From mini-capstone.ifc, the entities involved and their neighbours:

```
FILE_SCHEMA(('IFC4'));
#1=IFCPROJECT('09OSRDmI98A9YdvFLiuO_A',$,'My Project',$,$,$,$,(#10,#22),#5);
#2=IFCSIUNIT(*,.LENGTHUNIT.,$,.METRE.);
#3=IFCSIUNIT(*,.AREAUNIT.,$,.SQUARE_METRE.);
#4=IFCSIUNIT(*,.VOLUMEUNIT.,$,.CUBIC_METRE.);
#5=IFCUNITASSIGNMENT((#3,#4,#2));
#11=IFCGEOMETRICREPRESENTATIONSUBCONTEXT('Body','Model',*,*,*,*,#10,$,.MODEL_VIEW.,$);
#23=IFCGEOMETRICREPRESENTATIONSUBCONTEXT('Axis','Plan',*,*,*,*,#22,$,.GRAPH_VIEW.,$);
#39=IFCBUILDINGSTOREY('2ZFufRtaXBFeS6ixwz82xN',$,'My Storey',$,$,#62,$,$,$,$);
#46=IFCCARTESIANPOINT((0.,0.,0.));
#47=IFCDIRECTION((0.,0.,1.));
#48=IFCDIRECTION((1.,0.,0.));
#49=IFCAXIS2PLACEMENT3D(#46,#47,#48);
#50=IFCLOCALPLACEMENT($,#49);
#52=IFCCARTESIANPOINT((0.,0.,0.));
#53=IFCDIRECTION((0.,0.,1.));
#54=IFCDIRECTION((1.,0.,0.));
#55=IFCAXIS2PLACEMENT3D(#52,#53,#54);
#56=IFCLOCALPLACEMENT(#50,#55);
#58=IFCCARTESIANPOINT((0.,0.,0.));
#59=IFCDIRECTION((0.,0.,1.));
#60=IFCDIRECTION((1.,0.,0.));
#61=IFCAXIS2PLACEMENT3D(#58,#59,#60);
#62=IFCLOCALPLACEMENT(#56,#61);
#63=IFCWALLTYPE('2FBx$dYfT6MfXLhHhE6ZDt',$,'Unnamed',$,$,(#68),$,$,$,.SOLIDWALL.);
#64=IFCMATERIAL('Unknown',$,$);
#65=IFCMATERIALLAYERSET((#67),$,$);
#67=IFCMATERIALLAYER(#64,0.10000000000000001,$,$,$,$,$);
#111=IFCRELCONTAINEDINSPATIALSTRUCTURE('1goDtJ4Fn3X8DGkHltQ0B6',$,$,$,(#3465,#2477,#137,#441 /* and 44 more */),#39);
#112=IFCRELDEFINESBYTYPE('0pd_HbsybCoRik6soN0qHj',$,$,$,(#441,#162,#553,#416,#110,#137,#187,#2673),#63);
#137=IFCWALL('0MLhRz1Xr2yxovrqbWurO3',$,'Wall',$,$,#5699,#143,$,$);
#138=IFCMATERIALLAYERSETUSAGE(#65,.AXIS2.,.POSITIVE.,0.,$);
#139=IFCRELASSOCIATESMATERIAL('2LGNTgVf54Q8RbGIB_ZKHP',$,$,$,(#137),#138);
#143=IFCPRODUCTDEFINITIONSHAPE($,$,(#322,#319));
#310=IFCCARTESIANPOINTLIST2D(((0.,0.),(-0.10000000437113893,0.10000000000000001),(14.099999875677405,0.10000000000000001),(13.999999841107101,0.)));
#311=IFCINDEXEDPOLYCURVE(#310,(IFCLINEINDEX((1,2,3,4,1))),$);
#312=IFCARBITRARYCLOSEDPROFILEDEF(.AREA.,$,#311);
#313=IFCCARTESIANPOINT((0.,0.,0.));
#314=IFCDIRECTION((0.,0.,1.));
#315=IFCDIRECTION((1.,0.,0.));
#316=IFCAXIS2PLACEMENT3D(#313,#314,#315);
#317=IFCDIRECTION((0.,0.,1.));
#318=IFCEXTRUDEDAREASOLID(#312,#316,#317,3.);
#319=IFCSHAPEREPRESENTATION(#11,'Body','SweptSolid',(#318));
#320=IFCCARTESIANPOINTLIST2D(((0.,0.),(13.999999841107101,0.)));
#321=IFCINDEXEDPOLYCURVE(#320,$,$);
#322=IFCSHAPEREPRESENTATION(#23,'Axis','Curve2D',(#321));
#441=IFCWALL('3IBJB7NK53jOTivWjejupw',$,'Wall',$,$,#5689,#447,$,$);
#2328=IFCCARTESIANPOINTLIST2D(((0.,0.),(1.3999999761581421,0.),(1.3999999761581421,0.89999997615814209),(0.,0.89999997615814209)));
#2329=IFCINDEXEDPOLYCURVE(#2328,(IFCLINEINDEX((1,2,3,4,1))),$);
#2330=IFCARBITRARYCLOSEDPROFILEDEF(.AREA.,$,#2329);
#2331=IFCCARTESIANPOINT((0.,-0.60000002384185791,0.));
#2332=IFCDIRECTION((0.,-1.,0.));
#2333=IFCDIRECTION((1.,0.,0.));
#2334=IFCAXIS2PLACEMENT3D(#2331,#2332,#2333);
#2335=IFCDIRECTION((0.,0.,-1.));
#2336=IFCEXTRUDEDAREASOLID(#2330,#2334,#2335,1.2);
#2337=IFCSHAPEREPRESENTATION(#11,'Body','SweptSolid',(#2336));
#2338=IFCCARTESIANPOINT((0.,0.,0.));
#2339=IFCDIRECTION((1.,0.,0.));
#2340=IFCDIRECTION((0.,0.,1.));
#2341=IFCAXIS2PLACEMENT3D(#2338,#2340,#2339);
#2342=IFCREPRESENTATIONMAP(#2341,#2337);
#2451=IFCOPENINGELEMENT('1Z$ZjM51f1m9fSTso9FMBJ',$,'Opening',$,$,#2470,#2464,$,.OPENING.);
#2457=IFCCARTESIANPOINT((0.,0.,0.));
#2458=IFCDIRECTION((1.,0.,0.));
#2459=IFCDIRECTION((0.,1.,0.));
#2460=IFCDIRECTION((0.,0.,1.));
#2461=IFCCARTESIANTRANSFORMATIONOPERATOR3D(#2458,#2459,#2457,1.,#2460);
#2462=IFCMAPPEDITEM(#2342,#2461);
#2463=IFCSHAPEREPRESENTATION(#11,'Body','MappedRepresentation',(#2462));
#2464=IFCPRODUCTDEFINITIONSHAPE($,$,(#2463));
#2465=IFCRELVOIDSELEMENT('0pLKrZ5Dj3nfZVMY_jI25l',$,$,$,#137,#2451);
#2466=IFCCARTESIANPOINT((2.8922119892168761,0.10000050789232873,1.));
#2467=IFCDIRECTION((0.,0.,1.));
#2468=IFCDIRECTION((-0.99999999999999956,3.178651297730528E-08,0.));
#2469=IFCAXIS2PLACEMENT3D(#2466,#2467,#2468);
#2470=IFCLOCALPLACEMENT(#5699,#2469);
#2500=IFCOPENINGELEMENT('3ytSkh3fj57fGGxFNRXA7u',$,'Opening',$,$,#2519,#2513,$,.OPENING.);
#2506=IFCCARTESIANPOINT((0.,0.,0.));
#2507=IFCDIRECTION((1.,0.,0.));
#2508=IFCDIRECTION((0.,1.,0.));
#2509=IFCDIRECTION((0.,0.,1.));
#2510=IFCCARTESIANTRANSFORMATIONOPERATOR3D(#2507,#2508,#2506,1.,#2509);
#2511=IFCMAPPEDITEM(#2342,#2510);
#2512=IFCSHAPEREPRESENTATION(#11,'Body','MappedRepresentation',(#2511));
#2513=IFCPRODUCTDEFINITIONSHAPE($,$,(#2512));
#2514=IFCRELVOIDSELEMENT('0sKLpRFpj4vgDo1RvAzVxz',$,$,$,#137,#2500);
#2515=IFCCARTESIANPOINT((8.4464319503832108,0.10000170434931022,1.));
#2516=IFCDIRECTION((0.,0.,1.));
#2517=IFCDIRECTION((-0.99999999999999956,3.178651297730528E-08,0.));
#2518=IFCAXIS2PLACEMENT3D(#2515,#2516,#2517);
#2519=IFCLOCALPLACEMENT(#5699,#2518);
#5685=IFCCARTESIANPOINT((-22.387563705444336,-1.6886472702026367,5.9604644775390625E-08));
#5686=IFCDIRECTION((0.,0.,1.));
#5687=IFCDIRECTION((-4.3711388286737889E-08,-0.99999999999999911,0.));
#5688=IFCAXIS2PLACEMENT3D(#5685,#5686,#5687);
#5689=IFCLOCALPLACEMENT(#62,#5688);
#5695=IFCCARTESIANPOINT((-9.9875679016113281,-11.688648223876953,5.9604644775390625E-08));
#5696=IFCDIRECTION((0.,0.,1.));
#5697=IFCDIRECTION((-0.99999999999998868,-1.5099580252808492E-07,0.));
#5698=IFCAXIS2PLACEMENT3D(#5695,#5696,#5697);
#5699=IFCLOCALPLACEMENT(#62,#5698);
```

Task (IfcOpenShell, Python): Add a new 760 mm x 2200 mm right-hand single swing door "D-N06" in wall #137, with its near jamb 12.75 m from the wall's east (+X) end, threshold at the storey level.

```python
import numpy as np
import ifcopenshell
import ifcopenshell.api.feature
import ifcopenshell.api.geometry
import ifcopenshell.api.root
import ifcopenshell.api.spatial
import ifcopenshell.geom
import ifcopenshell.util.element
import ifcopenshell.util.placement
import ifcopenshell.util.representation
import ifcopenshell.util.shape
import ifcopenshell.util.unit

model = ifcopenshell.open("mini-capstone.ifc")
unit_scale = ifcopenshell.util.unit.calculate_unit_scale(model)
settings = ifcopenshell.geom.settings()


def volume(element):
    """Net volume in cubic metres, openings subtracted."""
    shape = ifcopenshell.geom.create_shape(settings, element)
    return ifcopenshell.util.shape.get_volume(shape.geometry)


wall = model.by_guid("0MLhRz1Xr2yxovrqbWurO3")
storey = ifcopenshell.util.element.get_container(wall, ifc_class="IfcBuildingStorey")
context = ifcopenshell.util.representation.get_context(model, "Model", "Body", "MODEL_VIEW")
before = volume(wall)

width, height, from_end, sill = 0.76, 2.2, 12.75, 0.0  # metres

# The wall runs along its own X axis, and the end named is its -X end.
wall_shape = ifcopenshell.geom.create_shape(settings, wall)
x, y, z = ifcopenshell.util.shape.get_vertices(wall_shape.geometry).T
start = x.min() + from_end
face, thickness = float(y.min()), float(y.max() - y.min())
wall_matrix = ifcopenshell.util.placement.get_local_placement(wall.ObjectPlacement)
level = ifcopenshell.util.placement.get_local_placement(storey.ObjectPlacement)[2, 3]


def in_wall(x, y):
    """Placement at x, y metres in the wall's axes, at sill height."""
    matrix = wall_matrix.copy()
    matrix[:, 3] = wall_matrix @ np.array([x / unit_scale, y / unit_scale, 0.0, 1.0])
    matrix[2, 3] = level + sill / unit_scale
    return matrix


# Opening: a box that overshoots both wall faces by 50 mm.
opening = ifcopenshell.api.root.create_entity(model, ifc_class="IfcOpeningElement", predefined_type="OPENING")
box = ifcopenshell.api.geometry.add_wall_representation(
    model, context=context, length=width, height=height, thickness=thickness + 0.1
)
ifcopenshell.api.geometry.assign_representation(model, product=opening, representation=box)
ifcopenshell.api.geometry.edit_object_placement(model, product=opening, matrix=in_wall(start, face - 0.05), is_si=False)
ifcopenshell.api.feature.add_feature(model, feature=opening, element=wall)

door = ifcopenshell.api.root.create_entity(model, ifc_class="IfcDoor", name="D-N06", predefined_type="DOOR")
door.OverallWidth, door.OverallHeight = width / unit_scale, height / unit_scale
door.OperationType = "SINGLE_SWING_RIGHT"
body = ifcopenshell.api.geometry.add_door_representation(
    model,
    context=context,
    overall_width=door.OverallWidth,
    overall_height=door.OverallHeight,
    operation_type="SINGLE_SWING_RIGHT",
    lining_properties={"LiningDepth": thickness / unit_scale, "ThresholdDepth": thickness / unit_scale},
)
ifcopenshell.api.geometry.assign_representation(model, product=door, representation=body)
ifcopenshell.api.spatial.assign_container(model, products=[door], relating_structure=storey)
ifcopenshell.api.feature.add_filling(model, opening=opening, element=door)

# The lining spans the wall, so the door starts at the wall face.
ifcopenshell.api.geometry.edit_object_placement(model, product=door, matrix=in_wall(start, face), is_si=False)

after = volume(wall)

print(f"wall volume {before:.3f} -> {after:.3f} m3")

model.write("mini-capstone-out.ifc")
```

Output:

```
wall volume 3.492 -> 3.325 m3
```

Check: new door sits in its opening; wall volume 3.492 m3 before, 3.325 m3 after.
